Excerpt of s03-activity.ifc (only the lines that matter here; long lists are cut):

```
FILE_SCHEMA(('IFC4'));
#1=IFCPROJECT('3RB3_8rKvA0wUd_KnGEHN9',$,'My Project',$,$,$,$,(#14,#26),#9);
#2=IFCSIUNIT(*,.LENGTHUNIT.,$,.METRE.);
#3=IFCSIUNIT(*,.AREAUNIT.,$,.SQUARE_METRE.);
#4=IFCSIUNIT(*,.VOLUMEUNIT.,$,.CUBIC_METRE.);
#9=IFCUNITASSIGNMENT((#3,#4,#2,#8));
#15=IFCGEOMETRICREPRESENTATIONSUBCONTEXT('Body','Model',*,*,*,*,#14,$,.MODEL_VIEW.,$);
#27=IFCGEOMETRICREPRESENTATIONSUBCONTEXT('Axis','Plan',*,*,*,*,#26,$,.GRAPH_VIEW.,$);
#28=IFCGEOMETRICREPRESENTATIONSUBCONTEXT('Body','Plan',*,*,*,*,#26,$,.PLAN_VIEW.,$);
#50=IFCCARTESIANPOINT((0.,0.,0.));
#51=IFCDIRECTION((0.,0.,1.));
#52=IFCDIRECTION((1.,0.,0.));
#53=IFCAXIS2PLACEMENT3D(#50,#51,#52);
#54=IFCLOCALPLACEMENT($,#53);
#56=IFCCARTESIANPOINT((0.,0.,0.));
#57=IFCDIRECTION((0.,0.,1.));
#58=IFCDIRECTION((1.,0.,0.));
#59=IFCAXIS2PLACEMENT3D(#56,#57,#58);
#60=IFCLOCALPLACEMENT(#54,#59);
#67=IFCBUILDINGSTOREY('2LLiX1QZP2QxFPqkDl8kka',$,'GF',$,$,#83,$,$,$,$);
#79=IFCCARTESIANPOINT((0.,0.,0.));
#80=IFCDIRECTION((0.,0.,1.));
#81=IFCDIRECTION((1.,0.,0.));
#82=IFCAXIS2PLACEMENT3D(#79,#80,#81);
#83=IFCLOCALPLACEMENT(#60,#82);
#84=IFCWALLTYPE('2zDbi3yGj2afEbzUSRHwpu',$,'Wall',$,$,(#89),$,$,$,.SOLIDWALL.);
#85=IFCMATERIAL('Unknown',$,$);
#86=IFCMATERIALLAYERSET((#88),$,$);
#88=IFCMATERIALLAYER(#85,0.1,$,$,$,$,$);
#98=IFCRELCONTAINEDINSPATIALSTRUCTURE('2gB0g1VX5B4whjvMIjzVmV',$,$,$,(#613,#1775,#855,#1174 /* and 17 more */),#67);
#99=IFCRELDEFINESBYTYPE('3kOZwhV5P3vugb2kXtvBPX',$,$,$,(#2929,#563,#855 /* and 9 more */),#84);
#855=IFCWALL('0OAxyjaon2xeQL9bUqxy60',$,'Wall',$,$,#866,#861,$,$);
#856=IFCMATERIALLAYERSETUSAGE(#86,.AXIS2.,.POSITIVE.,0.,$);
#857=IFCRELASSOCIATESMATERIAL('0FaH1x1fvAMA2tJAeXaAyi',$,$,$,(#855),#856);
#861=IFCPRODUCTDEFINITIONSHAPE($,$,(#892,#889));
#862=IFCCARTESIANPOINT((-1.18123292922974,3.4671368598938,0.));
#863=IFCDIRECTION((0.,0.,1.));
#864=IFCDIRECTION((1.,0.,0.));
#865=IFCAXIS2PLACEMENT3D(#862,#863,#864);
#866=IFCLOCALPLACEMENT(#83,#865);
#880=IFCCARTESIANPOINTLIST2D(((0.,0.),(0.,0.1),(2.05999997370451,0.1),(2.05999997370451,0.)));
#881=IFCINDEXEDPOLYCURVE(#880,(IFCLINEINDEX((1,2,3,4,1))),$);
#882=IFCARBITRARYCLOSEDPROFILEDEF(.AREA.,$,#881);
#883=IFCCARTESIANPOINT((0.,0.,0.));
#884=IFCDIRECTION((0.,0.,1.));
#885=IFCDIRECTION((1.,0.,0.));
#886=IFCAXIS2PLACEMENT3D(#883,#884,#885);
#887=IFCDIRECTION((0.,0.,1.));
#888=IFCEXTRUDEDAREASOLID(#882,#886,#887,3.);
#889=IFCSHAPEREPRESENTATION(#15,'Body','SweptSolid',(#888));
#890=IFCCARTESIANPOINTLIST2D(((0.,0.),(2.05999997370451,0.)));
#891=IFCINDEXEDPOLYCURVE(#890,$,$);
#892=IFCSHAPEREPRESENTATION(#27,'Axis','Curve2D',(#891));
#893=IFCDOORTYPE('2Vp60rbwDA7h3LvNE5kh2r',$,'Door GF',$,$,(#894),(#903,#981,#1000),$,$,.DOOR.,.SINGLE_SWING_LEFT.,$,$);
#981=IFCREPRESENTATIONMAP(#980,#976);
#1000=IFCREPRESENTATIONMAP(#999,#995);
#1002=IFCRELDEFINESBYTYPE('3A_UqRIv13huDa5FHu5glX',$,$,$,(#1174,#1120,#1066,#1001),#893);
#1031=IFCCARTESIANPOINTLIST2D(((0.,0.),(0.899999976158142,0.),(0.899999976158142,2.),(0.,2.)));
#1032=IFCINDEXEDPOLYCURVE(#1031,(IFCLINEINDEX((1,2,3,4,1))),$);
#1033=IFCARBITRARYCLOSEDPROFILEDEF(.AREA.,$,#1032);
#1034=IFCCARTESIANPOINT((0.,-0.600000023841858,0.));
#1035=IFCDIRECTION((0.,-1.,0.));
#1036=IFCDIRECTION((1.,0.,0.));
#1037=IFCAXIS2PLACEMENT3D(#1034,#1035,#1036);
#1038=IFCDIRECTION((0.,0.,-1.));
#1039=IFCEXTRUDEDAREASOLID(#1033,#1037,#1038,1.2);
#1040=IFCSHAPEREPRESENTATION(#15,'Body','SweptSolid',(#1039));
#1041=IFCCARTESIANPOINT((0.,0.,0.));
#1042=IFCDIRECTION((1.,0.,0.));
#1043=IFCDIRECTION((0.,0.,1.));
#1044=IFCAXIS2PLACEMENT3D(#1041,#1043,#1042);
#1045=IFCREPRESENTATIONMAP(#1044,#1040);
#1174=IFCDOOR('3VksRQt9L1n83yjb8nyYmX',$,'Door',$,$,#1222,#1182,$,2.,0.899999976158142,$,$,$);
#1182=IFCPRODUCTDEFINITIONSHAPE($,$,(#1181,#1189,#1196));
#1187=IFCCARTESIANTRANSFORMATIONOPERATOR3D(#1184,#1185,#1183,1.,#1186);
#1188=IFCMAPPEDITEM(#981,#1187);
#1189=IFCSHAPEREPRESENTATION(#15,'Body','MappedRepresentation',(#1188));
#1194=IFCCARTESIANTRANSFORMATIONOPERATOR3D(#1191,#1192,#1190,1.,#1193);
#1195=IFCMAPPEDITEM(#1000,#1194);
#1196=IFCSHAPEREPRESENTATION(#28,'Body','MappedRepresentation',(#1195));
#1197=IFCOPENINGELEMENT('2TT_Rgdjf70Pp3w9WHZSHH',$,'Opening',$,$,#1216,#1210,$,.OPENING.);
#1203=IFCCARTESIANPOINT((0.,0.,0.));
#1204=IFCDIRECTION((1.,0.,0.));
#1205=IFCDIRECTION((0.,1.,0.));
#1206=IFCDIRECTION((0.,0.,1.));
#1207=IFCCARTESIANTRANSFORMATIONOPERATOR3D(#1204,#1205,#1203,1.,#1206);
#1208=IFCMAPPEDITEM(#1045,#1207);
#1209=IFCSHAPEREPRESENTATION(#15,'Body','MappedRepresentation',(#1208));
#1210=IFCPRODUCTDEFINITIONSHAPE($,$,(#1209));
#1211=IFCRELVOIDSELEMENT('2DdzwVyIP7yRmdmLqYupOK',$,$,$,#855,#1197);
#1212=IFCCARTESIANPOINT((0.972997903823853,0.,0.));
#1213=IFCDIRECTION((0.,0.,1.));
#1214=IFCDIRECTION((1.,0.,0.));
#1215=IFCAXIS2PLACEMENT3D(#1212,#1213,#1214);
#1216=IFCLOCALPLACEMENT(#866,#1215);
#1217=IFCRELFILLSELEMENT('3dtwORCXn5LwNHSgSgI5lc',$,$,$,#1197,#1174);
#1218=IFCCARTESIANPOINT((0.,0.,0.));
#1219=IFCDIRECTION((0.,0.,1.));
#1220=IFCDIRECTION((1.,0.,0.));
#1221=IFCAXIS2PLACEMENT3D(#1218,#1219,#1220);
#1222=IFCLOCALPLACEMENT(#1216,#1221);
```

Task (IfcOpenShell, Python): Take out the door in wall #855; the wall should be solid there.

```python
import ifcopenshell
import ifcopenshell.api.feature
import ifcopenshell.api.root
import ifcopenshell.geom
import ifcopenshell.util.shape

model = ifcopenshell.open("s03-activity.ifc")
settings = ifcopenshell.geom.settings()


def volume(element):
    """Net volume in cubic metres, openings subtracted."""
    shape = ifcopenshell.geom.create_shape(settings, element)
    return ifcopenshell.util.shape.get_volume(shape.geometry)


door = model.by_guid("3VksRQt9L1n83yjb8nyYmX")
opening = door.FillsVoids[0].RelatingOpeningElement
wall = opening.VoidsElements[0].RelatingBuildingElement
before = volume(wall)

ifcopenshell.api.root.remove_product(model, product=door)
ifcopenshell.api.feature.remove_feature(model, feature=opening)

after = volume(wall)

print(f"wall volume {before:.3f} -> {after:.3f} m3")

model.write("s03-activity_v2.ifc")
```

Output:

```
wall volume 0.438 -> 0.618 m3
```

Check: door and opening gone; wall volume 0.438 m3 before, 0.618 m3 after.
